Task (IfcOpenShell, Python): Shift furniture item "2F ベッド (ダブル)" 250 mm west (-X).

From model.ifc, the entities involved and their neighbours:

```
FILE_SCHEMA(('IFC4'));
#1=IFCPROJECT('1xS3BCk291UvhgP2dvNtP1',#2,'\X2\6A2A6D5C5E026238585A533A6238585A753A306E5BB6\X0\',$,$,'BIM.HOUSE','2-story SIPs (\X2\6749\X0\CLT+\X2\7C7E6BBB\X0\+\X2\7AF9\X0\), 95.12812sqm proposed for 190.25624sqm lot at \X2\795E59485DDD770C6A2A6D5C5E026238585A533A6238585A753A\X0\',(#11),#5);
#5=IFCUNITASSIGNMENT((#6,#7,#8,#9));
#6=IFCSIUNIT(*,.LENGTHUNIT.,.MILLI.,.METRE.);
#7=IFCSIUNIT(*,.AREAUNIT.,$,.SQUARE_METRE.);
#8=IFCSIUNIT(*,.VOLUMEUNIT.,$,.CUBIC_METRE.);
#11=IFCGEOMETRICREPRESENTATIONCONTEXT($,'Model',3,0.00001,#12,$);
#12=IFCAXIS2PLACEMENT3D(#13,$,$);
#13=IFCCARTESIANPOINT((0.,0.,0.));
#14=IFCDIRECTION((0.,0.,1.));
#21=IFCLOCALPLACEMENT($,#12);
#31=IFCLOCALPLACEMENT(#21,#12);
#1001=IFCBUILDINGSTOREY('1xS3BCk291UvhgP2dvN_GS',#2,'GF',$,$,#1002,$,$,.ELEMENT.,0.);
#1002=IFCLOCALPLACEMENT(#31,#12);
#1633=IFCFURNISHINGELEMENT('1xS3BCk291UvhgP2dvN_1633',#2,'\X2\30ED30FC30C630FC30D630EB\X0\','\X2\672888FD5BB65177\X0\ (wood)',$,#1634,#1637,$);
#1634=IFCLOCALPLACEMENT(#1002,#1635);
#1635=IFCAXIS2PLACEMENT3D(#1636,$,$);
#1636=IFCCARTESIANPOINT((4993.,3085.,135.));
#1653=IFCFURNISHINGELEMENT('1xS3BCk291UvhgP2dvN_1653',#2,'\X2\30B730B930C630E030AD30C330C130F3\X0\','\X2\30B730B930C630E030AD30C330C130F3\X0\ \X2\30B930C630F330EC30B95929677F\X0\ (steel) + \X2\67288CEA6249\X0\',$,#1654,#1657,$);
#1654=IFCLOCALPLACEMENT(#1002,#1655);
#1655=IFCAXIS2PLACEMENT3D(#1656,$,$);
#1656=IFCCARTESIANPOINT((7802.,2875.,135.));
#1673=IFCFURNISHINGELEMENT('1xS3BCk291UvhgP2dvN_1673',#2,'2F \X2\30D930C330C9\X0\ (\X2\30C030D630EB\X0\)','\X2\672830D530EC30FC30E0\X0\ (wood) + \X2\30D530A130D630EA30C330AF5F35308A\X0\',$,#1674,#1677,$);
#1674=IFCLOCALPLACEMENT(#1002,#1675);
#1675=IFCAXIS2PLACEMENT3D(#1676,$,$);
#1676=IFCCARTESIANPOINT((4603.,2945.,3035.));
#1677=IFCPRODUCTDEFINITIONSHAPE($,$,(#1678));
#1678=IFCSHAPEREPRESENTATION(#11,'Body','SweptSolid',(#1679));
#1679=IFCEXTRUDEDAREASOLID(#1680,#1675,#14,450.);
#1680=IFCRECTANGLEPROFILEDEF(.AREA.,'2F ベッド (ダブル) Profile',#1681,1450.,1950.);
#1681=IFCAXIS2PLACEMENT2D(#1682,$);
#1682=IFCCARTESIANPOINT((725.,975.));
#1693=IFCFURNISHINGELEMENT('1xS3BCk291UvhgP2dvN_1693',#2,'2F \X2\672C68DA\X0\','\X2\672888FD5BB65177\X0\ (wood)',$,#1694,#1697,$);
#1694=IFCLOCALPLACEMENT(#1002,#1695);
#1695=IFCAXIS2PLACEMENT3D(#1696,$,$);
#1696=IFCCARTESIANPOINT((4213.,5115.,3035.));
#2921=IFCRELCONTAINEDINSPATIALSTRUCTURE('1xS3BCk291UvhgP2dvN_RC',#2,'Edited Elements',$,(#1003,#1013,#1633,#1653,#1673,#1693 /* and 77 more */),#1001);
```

```python
import ifcopenshell
import ifcopenshell.api.geometry
import ifcopenshell.util.placement

model = ifcopenshell.open("model.ifc")

item = model.by_guid("1xS3BCk291UvhgP2dvN_1673")
matrix = ifcopenshell.util.placement.get_local_placement(item.ObjectPlacement)
matrix[0, 3] -= 250.0
ifcopenshell.api.geometry.edit_object_placement(model, product=item, matrix=matrix, is_si=False)

print(ifcopenshell.util.placement.get_local_placement(item.ObjectPlacement).round(3) + 0.0)

model.write("model_updated.ifc")
```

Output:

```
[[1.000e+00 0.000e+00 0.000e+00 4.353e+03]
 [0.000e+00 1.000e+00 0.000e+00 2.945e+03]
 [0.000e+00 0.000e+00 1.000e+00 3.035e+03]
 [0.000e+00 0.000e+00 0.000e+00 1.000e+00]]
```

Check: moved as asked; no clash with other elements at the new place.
